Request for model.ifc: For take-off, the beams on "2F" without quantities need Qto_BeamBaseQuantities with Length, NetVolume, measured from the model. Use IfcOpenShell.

First a look at what the model holds.

```python
import ifcopenshell
import ifcopenshell.util.element
import ifcopenshell.util.unit

model = ifcopenshell.open("model.ifc")
print(model.schema)
for unit_type in ("LENGTHUNIT", "AREAUNIT", "VOLUMEUNIT"):
    print(unit_type, ifcopenshell.util.unit.calculate_unit_scale(model, unit_type))
storey = next(s for s in model.by_type("IfcBuildingStorey") if s.Name == "2F")
beams = [e for e in ifcopenshell.util.element.get_decomposition(storey) if e.is_a("IfcBeam")]
for e in sorted(beams, key=lambda e: e.id()):
    print(e.id(), e.is_a(), e.Name, list(ifcopenshell.util.element.get_psets(e, qtos_only=True)), sep=" | ")
```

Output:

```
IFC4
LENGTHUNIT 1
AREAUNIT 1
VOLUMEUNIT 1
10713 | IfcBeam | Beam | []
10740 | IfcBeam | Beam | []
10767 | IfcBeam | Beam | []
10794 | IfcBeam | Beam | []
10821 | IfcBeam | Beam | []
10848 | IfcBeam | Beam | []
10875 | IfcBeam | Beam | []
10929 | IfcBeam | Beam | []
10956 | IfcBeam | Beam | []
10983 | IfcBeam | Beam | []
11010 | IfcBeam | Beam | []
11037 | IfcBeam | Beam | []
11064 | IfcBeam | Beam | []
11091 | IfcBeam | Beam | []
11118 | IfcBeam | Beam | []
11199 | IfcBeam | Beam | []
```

```python
import ifcopenshell
import ifcopenshell.api.pset
import ifcopenshell.geom
import ifcopenshell.util.element
import ifcopenshell.util.shape
import ifcopenshell.util.unit

model = ifcopenshell.open("model.ifc")
unit_scale = ifcopenshell.util.unit.calculate_unit_scale(model)
volume_scale = ifcopenshell.util.unit.calculate_unit_scale(model, "VOLUMEUNIT")
settings = ifcopenshell.geom.settings()

storey = next(s for s in model.by_type("IfcBuildingStorey") if s.Name == "2F")
beams = [e for e in ifcopenshell.util.element.get_decomposition(storey) if e.is_a("IfcBeam")]

for e in sorted(beams, key=lambda e: e.id()):
    if ifcopenshell.util.element.get_psets(e, qtos_only=True, should_inherit=False):
        continue
    # Geometry comes back in metres, in the element's own axes.
    shape = ifcopenshell.geom.create_shape(settings, e)
    values = {
        "Length": ifcopenshell.util.shape.get_max_xyz(shape.geometry) / unit_scale,
        "NetVolume": ifcopenshell.util.shape.get_volume(shape.geometry) / volume_scale,
    }
    qto = ifcopenshell.api.pset.add_qto(model, product=e, name="Qto_BeamBaseQuantities")
    ifcopenshell.api.pset.edit_qto(model, qto=qto, properties=values)
    print(e.id(), {k: round(v, 3) for k, v in values.items()})

model.write("model_rev.ifc")
```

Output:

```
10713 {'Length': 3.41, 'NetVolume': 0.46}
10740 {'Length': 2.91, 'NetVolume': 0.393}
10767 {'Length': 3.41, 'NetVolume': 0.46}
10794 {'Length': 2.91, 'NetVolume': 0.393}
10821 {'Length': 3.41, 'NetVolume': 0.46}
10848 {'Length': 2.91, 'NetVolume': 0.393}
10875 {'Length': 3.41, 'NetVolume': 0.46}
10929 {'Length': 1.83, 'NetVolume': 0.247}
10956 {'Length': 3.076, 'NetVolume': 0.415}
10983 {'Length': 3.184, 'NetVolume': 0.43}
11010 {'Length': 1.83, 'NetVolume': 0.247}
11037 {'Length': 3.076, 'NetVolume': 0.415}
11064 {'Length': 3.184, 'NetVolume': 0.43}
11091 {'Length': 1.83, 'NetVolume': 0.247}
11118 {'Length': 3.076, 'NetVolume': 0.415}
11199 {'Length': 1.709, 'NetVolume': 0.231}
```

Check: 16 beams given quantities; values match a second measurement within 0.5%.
